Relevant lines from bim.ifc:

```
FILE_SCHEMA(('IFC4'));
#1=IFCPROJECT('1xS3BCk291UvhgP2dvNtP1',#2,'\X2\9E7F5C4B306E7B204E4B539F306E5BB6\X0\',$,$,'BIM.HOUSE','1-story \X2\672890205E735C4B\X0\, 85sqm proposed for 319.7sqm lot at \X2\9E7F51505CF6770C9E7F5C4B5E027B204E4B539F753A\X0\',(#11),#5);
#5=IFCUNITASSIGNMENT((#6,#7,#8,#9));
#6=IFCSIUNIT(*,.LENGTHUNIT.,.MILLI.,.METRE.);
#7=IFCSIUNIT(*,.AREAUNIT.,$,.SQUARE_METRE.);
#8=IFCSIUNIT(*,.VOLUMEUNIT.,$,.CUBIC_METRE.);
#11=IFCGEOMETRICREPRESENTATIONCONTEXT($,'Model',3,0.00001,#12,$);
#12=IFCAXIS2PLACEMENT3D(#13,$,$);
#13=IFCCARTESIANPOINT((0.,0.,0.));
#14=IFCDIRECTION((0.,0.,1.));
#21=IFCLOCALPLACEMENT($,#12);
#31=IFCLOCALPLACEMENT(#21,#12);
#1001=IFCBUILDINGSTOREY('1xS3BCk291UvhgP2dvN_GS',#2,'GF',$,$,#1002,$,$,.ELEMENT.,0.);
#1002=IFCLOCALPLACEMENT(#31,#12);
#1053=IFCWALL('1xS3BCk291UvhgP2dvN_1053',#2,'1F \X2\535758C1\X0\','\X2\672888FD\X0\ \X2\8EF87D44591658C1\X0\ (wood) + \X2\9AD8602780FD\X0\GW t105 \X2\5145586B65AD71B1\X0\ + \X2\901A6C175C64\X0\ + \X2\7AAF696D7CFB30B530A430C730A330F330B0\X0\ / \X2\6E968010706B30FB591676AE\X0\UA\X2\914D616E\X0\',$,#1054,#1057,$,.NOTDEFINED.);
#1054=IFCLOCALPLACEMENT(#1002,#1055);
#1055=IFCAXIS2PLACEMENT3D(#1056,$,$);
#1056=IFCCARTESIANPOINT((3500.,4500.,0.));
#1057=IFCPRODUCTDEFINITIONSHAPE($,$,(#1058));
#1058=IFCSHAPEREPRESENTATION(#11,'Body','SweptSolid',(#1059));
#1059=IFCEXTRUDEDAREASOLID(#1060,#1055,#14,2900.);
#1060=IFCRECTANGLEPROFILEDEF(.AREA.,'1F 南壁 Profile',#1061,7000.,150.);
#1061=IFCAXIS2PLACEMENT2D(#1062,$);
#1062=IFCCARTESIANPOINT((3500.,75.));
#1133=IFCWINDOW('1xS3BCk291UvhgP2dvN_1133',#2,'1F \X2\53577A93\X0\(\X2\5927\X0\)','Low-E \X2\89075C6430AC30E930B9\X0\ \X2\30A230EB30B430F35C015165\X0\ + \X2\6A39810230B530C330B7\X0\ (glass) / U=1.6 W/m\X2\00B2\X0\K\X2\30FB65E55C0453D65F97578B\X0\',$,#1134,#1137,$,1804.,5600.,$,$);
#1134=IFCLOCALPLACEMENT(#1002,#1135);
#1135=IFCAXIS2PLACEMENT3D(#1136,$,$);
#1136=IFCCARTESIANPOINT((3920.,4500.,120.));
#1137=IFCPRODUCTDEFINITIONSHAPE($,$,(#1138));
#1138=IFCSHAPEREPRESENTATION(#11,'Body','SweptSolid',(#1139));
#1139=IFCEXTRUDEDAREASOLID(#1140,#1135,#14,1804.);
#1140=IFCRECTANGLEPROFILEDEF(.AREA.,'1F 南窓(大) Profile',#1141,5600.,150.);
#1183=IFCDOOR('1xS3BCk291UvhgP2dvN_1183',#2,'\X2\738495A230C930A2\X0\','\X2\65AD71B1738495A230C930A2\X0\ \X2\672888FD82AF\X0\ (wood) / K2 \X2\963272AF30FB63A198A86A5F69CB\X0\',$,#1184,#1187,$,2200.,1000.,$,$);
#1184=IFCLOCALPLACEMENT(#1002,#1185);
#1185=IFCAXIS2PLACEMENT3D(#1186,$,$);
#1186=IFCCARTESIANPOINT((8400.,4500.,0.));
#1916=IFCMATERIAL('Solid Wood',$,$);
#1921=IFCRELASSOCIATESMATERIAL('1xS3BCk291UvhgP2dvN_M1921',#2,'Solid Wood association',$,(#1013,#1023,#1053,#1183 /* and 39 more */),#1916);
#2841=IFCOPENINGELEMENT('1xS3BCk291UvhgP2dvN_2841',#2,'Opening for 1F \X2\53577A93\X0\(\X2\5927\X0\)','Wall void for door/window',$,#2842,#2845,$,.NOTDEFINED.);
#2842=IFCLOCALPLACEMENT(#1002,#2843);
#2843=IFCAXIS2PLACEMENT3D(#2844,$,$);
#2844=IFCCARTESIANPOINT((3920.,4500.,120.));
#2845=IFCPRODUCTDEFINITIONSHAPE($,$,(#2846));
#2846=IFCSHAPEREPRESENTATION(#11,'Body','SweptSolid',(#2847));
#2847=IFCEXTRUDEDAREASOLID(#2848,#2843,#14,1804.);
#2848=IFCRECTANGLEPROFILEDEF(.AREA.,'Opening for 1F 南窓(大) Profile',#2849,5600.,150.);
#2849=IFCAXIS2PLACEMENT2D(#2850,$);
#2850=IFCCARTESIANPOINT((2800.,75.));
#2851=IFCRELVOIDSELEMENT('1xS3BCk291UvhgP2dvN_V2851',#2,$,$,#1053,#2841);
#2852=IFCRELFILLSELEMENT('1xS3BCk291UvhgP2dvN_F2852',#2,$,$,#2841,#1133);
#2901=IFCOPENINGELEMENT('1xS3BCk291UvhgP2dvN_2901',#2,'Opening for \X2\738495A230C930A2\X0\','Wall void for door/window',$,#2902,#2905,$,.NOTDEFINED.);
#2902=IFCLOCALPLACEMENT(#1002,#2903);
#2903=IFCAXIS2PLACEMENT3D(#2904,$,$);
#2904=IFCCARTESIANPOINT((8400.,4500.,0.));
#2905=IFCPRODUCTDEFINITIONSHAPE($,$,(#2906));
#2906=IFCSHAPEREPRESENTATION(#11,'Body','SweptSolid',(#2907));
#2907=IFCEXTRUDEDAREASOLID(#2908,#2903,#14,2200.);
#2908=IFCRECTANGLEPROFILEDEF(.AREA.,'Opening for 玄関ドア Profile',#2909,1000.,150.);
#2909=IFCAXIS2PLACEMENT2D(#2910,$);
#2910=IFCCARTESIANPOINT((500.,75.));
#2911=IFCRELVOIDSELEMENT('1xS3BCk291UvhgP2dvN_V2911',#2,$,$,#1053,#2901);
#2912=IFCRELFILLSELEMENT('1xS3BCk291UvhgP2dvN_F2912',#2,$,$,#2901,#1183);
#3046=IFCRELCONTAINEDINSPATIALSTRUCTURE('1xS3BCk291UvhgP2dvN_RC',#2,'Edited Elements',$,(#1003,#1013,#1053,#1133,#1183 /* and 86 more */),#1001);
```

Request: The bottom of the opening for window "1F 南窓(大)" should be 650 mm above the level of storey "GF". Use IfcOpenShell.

```python
import numpy as np
import ifcopenshell
import ifcopenshell.api.geometry
import ifcopenshell.geom
import ifcopenshell.util.element
import ifcopenshell.util.placement
import ifcopenshell.util.shape
import ifcopenshell.util.unit

model = ifcopenshell.open("bim.ifc")
unit_scale = ifcopenshell.util.unit.calculate_unit_scale(model)

window = model.by_id(1133)
opening = window.FillsVoids[0].RelatingOpeningElement
storey = ifcopenshell.util.element.get_container(window, ifc_class="IfcBuildingStorey")
level = ifcopenshell.util.placement.get_local_placement(storey.ObjectPlacement)[2, 3]

# The opening's origin need not be at the sill, so measure its lowest point.
shape = ifcopenshell.geom.create_shape(ifcopenshell.geom.settings(), opening)
bottom = ifcopenshell.util.shape.get_shape_bottom_elevation(shape, shape.geometry) / unit_scale
dz = level + 0.65 / unit_scale - bottom

shift = np.array([0.0, 0.0, dz])
# The window is not placed relative to its opening, so move both.
for product in (opening, window):
    matrix = ifcopenshell.util.placement.get_local_placement(product.ObjectPlacement)
    matrix[:3, 3] += shift
    ifcopenshell.api.geometry.edit_object_placement(model, product=product, matrix=matrix, is_si=False)

print(f"moved by {dz * unit_scale:+.3f} m")

model.write("bim_v2.ifc")
```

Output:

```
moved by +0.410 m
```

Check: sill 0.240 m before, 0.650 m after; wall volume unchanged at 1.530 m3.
